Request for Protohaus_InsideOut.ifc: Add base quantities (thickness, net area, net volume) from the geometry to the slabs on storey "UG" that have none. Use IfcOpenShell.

First a look at what the model holds.

```python
import ifcopenshell
import ifcopenshell.util.element
import ifcopenshell.util.unit

model = ifcopenshell.open("Protohaus_InsideOut.ifc")
print(model.schema)
for unit_type in ("LENGTHUNIT", "AREAUNIT", "VOLUMEUNIT"):
    print(unit_type, ifcopenshell.util.unit.calculate_unit_scale(model, unit_type))
storey = next(s for s in model.by_type("IfcBuildingStorey") if s.Name == "UG")
slabs = [e for e in ifcopenshell.util.element.get_decomposition(storey) if e.is_a("IfcSlab")]
for e in sorted(slabs, key=lambda e: e.id()):
    print(e.id(), e.is_a(), e.Name, list(ifcopenshell.util.element.get_psets(e, qtos_only=True)), sep=" | ")
```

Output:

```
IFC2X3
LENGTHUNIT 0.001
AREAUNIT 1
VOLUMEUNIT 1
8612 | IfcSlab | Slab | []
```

```python
import ifcopenshell
import ifcopenshell.api.pset
import ifcopenshell.geom
import ifcopenshell.util.element
import ifcopenshell.util.shape
import ifcopenshell.util.unit

model = ifcopenshell.open("Protohaus_InsideOut.ifc")
unit_scale = ifcopenshell.util.unit.calculate_unit_scale(model)
area_scale = ifcopenshell.util.unit.calculate_unit_scale(model, "AREAUNIT")
volume_scale = ifcopenshell.util.unit.calculate_unit_scale(model, "VOLUMEUNIT")
settings = ifcopenshell.geom.settings()

storey = next(s for s in model.by_type("IfcBuildingStorey") if s.Name == "UG")
slabs = [e for e in ifcopenshell.util.element.get_decomposition(storey) if e.is_a("IfcSlab")]

for e in sorted(slabs, key=lambda e: e.id()):
    if ifcopenshell.util.element.get_psets(e, qtos_only=True, should_inherit=False):
        continue
    # Geometry comes back in metres, in the element's own axes.
    shape = ifcopenshell.geom.create_shape(settings, e)
    values = {
        "Width": ifcopenshell.util.shape.get_z(shape.geometry) / unit_scale,
        "NetArea": ifcopenshell.util.shape.get_footprint_area(shape.geometry) / area_scale,
        "NetVolume": ifcopenshell.util.shape.get_volume(shape.geometry) / volume_scale,
    }
    qto = ifcopenshell.api.pset.add_qto(model, product=e, name="BaseQuantities")
    ifcopenshell.api.pset.edit_qto(model, qto=qto, properties=values)
    print(e.id(), {k: round(v, 3) for k, v in values.items()})

model.write("Protohaus_InsideOut_rev.ifc")
```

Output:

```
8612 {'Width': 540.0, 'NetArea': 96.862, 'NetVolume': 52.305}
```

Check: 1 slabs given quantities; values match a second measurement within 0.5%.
